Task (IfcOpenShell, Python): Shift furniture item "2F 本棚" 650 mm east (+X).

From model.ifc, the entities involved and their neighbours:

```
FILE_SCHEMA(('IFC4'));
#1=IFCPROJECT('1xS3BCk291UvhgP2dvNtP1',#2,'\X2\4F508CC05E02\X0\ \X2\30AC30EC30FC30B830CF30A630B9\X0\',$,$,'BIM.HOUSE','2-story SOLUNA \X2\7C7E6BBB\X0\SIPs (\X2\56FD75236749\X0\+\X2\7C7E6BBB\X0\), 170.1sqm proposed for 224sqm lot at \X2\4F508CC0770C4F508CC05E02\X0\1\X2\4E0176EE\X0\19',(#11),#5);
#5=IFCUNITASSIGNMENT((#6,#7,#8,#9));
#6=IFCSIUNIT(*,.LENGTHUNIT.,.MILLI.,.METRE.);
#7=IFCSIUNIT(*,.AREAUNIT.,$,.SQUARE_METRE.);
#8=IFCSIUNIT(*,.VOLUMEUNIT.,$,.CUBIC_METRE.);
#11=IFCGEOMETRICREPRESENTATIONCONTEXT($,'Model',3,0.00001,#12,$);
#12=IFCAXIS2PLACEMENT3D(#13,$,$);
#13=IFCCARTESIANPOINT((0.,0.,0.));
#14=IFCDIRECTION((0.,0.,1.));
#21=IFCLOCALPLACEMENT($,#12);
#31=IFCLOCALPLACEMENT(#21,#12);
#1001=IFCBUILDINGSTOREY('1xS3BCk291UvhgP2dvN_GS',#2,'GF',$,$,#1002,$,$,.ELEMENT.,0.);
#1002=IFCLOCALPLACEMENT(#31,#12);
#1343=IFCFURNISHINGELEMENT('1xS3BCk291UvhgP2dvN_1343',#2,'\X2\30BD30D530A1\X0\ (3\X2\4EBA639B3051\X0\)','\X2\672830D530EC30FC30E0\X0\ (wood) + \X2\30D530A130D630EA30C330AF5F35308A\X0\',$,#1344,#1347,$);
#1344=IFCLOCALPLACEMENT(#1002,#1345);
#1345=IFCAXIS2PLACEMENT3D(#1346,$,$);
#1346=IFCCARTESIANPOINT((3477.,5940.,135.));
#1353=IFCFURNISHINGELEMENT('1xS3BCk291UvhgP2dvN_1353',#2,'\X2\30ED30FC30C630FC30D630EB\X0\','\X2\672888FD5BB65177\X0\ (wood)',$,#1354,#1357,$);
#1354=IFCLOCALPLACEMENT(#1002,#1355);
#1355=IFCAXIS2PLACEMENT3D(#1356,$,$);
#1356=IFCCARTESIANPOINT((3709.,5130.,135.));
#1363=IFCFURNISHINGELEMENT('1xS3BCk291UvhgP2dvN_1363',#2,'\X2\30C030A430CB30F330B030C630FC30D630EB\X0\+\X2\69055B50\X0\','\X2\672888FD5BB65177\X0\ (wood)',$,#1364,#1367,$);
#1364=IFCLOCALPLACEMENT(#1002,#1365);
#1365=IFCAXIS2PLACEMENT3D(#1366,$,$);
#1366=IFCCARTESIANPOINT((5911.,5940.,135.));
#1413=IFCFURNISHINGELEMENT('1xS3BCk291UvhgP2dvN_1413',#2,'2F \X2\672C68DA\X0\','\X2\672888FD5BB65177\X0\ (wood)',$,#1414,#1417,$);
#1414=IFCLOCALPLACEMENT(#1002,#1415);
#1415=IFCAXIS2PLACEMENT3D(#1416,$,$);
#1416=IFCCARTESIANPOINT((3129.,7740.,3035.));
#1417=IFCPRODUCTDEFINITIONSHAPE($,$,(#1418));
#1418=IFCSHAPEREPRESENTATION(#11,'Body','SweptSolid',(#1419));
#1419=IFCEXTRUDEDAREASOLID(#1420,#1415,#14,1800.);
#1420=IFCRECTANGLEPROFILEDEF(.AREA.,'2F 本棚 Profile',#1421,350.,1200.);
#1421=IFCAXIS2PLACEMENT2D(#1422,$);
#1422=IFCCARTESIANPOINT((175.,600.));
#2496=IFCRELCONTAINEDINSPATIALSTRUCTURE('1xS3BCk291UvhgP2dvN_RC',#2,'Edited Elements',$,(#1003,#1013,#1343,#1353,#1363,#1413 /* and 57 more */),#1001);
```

```python
import ifcopenshell
import ifcopenshell.api.geometry
import ifcopenshell.util.placement
import ifcopenshell.util.unit

model = ifcopenshell.open("model.ifc")
unit_scale = ifcopenshell.util.unit.calculate_unit_scale(model)

item = model.by_guid("1xS3BCk291UvhgP2dvN_1413")
matrix = ifcopenshell.util.placement.get_local_placement(item.ObjectPlacement)
matrix[0, 3] += 0.65 / unit_scale
ifcopenshell.api.geometry.edit_object_placement(model, product=item, matrix=matrix, is_si=False)

print(ifcopenshell.util.placement.get_local_placement(item.ObjectPlacement).round(3) + 0.0)

model.write("model_edited.ifc")
```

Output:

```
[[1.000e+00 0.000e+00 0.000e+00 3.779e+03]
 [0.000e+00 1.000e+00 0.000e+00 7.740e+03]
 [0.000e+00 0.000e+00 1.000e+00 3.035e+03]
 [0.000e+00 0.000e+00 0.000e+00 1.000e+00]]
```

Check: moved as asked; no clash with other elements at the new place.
